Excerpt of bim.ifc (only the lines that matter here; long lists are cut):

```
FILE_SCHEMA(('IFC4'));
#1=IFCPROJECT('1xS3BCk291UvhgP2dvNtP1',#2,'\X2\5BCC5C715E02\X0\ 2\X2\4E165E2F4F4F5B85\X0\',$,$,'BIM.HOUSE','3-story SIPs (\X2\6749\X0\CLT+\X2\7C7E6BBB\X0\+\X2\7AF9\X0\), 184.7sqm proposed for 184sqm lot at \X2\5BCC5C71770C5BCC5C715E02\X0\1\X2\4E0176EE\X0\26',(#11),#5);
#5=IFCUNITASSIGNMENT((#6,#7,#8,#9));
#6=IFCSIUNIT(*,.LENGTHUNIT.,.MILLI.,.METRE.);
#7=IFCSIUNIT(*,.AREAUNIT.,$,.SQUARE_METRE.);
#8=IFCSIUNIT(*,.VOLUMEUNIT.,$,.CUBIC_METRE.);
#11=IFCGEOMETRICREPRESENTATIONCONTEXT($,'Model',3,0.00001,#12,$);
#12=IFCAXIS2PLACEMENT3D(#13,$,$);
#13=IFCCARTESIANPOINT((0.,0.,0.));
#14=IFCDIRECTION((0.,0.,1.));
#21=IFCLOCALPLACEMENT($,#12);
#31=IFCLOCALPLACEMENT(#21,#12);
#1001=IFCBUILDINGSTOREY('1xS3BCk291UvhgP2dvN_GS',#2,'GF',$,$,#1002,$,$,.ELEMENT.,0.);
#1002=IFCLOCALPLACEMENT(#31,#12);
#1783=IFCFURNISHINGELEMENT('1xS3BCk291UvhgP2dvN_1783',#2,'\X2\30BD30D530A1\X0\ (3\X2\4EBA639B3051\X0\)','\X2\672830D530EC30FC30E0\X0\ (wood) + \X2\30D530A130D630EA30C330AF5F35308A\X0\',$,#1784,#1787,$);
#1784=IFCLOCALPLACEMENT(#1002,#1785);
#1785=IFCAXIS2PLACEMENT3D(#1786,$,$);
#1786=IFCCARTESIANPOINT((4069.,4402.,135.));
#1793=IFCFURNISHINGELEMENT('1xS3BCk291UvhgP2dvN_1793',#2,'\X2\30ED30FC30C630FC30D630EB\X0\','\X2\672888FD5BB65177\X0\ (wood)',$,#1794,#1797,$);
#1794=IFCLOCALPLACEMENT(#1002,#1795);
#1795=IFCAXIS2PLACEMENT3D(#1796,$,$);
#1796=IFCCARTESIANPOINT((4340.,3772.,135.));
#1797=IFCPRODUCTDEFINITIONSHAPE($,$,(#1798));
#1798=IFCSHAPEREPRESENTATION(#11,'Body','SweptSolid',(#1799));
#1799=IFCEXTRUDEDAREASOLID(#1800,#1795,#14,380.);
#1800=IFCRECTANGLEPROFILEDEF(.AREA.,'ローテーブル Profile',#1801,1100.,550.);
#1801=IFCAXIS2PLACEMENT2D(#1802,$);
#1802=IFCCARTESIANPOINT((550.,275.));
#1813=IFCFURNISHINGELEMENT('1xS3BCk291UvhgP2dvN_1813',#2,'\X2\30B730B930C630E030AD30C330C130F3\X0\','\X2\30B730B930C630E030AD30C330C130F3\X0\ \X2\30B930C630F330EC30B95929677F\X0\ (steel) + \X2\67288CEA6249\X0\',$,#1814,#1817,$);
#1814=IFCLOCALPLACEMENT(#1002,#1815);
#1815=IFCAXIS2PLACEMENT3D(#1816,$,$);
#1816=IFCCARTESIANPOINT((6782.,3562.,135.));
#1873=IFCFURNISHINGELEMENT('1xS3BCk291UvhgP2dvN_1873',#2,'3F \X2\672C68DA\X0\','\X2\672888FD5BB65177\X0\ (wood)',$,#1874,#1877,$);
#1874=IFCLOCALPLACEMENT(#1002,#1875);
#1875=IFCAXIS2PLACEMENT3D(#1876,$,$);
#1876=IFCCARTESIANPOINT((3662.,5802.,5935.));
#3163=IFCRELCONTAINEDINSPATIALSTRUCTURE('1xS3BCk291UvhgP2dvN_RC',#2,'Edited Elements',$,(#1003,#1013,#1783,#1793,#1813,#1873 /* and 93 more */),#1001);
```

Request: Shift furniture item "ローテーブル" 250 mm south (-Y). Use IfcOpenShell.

```python
import ifcopenshell
import ifcopenshell.api.geometry
import ifcopenshell.util.placement
import ifcopenshell.util.unit

model = ifcopenshell.open("bim.ifc")
unit_scale = ifcopenshell.util.unit.calculate_unit_scale(model)

item = model.by_guid("1xS3BCk291UvhgP2dvN_1793")
matrix = ifcopenshell.util.placement.get_local_placement(item.ObjectPlacement)
matrix[1, 3] -= 0.25 / unit_scale
ifcopenshell.api.geometry.edit_object_placement(model, product=item, matrix=matrix, is_si=False)

print(ifcopenshell.util.placement.get_local_placement(item.ObjectPlacement).round(3) + 0.0)

model.write("bim_v2.ifc")
```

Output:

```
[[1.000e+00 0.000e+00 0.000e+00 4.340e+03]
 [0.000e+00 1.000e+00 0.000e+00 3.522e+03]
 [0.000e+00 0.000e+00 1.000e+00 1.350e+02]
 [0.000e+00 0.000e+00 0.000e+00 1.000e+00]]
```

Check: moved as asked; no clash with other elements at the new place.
